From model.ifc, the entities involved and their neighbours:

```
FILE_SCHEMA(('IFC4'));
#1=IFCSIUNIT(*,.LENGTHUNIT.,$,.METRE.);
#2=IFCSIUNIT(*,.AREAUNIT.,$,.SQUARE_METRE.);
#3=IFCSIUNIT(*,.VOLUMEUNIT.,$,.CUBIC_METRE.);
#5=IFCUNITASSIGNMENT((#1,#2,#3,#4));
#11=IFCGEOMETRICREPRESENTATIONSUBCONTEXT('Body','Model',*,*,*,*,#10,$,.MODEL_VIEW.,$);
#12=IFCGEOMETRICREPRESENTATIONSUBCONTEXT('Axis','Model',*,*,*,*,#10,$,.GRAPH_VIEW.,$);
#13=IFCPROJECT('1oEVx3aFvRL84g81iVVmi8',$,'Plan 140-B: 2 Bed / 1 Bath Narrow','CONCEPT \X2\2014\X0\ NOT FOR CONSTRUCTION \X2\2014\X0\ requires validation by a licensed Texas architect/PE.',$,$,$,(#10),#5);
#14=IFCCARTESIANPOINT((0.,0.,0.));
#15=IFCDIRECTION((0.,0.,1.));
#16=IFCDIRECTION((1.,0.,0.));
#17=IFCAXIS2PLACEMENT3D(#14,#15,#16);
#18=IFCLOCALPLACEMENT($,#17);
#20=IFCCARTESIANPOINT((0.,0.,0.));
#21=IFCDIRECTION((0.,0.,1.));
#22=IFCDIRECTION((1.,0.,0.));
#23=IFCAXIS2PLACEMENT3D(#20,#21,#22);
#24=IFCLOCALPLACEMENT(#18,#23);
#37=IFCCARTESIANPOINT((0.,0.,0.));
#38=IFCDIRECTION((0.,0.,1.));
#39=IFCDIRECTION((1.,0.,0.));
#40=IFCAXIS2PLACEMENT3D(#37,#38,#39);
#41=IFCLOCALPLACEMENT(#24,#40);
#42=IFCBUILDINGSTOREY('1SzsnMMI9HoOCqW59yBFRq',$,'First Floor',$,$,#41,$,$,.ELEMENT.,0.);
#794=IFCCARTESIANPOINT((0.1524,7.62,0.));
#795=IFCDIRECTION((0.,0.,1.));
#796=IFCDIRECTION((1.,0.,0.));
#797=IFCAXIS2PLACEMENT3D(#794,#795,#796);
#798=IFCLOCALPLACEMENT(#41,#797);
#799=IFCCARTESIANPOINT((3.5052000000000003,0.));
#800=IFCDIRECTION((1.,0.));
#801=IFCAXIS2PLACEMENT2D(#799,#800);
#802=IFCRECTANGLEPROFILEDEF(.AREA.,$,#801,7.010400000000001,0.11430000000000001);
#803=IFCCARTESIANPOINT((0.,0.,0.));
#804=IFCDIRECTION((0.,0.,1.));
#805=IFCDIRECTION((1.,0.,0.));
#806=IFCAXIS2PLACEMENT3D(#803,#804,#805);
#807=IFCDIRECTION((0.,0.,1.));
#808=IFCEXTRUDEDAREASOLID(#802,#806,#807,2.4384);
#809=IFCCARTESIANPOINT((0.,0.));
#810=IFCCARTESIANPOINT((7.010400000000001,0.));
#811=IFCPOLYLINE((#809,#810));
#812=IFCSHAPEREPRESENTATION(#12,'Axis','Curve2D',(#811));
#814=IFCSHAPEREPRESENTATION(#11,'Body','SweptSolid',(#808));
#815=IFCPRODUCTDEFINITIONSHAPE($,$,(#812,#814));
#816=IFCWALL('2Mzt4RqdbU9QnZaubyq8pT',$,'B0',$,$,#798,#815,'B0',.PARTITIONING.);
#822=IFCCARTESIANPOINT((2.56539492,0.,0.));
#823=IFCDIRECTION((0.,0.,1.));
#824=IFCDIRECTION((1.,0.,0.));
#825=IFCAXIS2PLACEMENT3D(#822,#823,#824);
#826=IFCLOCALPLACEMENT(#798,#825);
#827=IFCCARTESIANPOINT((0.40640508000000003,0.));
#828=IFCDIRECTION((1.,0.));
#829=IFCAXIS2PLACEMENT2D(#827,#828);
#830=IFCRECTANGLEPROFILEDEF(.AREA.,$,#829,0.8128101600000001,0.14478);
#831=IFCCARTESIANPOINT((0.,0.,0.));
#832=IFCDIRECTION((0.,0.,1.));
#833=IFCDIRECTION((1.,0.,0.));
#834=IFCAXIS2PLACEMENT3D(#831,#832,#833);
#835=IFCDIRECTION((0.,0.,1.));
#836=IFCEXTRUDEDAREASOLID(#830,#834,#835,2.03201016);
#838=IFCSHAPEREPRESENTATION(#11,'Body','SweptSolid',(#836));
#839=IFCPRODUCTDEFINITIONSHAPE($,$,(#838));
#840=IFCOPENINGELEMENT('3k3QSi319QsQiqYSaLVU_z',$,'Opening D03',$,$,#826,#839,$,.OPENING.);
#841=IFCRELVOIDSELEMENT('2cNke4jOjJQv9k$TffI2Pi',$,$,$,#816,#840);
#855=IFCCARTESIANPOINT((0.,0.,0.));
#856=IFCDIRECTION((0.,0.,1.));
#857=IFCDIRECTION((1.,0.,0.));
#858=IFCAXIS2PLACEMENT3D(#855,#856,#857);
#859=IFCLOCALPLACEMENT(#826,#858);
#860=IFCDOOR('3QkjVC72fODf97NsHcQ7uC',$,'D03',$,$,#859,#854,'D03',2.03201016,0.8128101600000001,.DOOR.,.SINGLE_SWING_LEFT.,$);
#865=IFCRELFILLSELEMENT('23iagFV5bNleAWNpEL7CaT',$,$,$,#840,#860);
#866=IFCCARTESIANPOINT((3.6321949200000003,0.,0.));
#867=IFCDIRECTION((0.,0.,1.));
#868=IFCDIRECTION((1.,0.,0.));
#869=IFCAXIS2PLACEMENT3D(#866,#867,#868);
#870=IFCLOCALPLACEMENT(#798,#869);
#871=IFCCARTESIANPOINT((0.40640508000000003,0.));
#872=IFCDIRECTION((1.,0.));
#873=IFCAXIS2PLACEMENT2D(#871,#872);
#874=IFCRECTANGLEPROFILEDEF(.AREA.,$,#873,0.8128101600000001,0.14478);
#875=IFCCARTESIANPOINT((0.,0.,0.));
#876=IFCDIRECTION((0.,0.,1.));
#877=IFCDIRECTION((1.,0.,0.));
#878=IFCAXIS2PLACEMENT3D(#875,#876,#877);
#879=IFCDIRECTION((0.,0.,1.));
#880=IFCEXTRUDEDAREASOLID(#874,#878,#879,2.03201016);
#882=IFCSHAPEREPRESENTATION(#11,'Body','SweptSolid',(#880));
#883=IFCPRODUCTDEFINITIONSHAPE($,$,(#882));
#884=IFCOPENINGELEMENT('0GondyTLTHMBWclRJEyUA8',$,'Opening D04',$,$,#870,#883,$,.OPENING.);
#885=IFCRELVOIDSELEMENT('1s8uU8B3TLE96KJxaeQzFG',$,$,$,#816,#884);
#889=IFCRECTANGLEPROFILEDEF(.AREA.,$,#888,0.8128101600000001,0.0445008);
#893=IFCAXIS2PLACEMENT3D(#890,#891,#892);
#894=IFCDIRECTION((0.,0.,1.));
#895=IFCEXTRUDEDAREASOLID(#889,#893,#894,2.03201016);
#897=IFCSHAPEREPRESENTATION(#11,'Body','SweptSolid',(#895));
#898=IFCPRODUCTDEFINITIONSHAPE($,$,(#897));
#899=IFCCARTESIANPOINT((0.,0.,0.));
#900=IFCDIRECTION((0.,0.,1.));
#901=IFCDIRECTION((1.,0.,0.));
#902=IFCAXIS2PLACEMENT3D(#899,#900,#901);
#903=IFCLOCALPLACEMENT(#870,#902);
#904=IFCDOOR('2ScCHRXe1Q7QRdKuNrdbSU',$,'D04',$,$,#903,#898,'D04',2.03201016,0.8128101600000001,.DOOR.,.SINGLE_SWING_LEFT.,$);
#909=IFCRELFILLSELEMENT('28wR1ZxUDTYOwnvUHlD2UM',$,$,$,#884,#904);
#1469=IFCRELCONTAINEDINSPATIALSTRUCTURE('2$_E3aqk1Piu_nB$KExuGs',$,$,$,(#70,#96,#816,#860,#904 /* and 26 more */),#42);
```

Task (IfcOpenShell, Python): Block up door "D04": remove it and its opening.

```python
import ifcopenshell
import ifcopenshell.api.feature
import ifcopenshell.api.root
import ifcopenshell.geom
import ifcopenshell.util.shape

model = ifcopenshell.open("model.ifc")
settings = ifcopenshell.geom.settings()


def volume(element):
    """Net volume in cubic metres, openings subtracted."""
    shape = ifcopenshell.geom.create_shape(settings, element)
    return ifcopenshell.util.shape.get_volume(shape.geometry)


door = model.by_id(904)
opening = door.FillsVoids[0].RelatingOpeningElement
wall = opening.VoidsElements[0].RelatingBuildingElement
before = volume(wall)

ifcopenshell.api.root.remove_product(model, product=door)
ifcopenshell.api.feature.remove_feature(model, feature=opening)

after = volume(wall)

print(f"wall volume {before:.3f} -> {after:.3f} m3")

model.write("model_edited.ifc")
```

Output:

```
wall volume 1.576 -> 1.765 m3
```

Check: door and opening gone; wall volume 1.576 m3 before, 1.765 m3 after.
